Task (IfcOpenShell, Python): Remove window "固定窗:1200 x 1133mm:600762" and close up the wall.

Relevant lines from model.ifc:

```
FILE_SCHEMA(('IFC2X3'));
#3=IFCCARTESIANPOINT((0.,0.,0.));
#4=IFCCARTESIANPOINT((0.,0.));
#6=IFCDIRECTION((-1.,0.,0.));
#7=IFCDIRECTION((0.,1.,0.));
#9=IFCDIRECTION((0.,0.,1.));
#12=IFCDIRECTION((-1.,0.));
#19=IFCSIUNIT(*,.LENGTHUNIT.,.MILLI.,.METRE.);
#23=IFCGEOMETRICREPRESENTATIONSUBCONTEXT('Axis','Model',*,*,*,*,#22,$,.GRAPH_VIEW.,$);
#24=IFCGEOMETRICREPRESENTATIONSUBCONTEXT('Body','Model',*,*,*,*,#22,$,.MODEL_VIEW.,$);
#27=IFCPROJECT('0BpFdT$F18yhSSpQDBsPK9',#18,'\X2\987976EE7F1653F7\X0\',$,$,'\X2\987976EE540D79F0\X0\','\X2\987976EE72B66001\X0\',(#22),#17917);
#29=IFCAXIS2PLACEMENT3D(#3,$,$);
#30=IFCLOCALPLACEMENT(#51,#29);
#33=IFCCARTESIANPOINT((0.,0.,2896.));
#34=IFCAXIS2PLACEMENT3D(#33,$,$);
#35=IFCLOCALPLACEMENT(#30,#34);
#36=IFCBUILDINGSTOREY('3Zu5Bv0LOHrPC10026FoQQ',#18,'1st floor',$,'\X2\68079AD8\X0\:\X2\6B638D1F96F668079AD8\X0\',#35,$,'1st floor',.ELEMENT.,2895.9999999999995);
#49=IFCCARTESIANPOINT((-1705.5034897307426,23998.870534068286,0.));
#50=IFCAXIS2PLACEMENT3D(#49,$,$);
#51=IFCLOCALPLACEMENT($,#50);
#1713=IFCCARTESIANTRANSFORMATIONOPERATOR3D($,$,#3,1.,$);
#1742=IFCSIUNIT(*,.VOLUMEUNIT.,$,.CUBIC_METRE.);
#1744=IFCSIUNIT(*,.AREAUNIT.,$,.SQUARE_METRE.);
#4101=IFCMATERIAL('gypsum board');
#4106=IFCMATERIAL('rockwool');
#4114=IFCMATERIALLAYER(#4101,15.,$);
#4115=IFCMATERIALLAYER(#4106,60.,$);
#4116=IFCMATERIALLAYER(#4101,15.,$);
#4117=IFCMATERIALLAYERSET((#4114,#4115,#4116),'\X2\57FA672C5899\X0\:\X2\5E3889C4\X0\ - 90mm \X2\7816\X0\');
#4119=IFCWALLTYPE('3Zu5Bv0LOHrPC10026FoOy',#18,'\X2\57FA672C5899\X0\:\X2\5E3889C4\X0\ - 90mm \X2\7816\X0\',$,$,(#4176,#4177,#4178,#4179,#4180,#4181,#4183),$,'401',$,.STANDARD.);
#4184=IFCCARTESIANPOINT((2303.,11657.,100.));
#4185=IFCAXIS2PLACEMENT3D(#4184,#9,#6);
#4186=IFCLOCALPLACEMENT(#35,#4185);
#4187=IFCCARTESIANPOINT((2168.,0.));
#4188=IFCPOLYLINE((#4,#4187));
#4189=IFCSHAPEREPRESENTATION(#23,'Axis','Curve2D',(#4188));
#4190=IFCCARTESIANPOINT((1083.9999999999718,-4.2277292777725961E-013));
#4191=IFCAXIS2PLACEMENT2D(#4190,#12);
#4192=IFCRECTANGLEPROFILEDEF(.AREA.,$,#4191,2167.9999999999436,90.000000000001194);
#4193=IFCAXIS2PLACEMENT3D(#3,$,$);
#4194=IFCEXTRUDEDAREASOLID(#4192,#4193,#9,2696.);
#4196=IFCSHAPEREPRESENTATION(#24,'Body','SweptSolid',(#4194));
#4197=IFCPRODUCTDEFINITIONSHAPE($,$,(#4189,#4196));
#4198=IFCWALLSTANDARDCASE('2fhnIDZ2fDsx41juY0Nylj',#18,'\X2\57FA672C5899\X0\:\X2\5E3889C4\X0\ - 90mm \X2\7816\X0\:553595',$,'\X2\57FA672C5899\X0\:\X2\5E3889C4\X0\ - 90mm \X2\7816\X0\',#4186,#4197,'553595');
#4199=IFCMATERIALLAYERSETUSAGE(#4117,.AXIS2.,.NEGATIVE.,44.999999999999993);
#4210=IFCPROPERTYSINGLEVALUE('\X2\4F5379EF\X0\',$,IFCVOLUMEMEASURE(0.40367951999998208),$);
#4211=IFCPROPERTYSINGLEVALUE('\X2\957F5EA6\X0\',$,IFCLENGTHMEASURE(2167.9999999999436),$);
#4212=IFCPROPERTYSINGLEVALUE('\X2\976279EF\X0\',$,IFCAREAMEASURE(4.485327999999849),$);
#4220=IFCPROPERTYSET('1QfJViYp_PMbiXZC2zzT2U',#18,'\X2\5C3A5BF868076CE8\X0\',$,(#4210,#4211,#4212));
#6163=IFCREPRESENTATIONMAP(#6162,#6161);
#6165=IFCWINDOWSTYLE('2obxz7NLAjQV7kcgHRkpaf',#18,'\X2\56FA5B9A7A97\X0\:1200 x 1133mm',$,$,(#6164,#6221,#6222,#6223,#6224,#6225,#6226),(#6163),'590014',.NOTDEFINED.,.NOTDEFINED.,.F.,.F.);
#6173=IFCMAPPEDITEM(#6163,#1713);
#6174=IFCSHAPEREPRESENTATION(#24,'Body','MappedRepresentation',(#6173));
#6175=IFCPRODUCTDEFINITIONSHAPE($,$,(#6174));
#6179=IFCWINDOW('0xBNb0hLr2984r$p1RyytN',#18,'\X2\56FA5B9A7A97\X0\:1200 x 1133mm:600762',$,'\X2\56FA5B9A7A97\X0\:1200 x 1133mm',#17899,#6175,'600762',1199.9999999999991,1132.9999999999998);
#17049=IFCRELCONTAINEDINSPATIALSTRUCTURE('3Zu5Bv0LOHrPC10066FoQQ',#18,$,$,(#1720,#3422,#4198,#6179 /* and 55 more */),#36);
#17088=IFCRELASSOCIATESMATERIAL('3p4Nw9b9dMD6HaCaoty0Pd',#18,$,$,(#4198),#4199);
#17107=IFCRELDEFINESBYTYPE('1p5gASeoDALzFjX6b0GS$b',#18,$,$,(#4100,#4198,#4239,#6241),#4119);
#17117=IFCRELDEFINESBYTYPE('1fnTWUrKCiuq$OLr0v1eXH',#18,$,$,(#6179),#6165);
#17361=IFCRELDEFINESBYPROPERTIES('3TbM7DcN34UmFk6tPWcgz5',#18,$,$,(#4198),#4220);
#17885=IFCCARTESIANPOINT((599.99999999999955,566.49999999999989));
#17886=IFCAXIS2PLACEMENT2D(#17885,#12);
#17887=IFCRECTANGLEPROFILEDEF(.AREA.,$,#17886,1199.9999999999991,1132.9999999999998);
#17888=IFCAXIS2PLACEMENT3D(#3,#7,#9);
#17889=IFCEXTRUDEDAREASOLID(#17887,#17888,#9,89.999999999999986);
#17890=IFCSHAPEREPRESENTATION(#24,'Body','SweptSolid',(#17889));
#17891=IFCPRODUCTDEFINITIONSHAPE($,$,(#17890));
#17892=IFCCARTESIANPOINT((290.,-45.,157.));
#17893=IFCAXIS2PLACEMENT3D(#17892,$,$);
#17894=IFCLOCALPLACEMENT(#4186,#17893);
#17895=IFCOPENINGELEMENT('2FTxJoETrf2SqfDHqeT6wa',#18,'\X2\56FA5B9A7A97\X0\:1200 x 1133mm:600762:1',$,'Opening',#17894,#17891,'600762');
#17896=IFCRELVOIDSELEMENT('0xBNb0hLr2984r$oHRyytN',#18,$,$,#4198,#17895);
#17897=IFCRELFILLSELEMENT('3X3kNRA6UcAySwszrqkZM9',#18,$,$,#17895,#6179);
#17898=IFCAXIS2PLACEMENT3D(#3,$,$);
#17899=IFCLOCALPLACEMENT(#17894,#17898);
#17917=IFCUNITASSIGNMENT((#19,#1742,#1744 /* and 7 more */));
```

```python
import ifcopenshell
import ifcopenshell.api.feature
import ifcopenshell.api.pset
import ifcopenshell.api.root
import ifcopenshell.geom
import ifcopenshell.util.element
import ifcopenshell.util.shape
import ifcopenshell.util.unit

model = ifcopenshell.open("model.ifc")
area_scale = ifcopenshell.util.unit.calculate_unit_scale(model, "AREAUNIT")
volume_scale = ifcopenshell.util.unit.calculate_unit_scale(model, "VOLUMEUNIT")
settings = ifcopenshell.geom.settings()


def volume(element):
    """Net volume in cubic metres, openings subtracted."""
    shape = ifcopenshell.geom.create_shape(settings, element)
    return ifcopenshell.util.shape.get_volume(shape.geometry)


window = model.by_guid("0xBNb0hLr2984r$p1RyytN")
opening = window.FillsVoids[0].RelatingOpeningElement
wall = opening.VoidsElements[0].RelatingBuildingElement
before = volume(wall)

ifcopenshell.api.root.remove_product(model, product=window)
ifcopenshell.api.feature.remove_feature(model, feature=opening)

after = volume(wall)
thickness = 0.09  # wall thickness in metres

# Update the wall's stored quantities.
pset = model.by_id(ifcopenshell.util.element.get_pset(wall, "尺寸标注", should_inherit=False)["id"])
ifcopenshell.api.pset.edit_pset(model, pset=pset, properties={
    "体积": model.create_entity("IfcVolumeMeasure", after / volume_scale),
    "面积": model.create_entity("IfcAreaMeasure", after / thickness / area_scale),
})

print(f"wall volume {before:.3f} -> {after:.3f} m3")

model.write("model_edited.ifc")
```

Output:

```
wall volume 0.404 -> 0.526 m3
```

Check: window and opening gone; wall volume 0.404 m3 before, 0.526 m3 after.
